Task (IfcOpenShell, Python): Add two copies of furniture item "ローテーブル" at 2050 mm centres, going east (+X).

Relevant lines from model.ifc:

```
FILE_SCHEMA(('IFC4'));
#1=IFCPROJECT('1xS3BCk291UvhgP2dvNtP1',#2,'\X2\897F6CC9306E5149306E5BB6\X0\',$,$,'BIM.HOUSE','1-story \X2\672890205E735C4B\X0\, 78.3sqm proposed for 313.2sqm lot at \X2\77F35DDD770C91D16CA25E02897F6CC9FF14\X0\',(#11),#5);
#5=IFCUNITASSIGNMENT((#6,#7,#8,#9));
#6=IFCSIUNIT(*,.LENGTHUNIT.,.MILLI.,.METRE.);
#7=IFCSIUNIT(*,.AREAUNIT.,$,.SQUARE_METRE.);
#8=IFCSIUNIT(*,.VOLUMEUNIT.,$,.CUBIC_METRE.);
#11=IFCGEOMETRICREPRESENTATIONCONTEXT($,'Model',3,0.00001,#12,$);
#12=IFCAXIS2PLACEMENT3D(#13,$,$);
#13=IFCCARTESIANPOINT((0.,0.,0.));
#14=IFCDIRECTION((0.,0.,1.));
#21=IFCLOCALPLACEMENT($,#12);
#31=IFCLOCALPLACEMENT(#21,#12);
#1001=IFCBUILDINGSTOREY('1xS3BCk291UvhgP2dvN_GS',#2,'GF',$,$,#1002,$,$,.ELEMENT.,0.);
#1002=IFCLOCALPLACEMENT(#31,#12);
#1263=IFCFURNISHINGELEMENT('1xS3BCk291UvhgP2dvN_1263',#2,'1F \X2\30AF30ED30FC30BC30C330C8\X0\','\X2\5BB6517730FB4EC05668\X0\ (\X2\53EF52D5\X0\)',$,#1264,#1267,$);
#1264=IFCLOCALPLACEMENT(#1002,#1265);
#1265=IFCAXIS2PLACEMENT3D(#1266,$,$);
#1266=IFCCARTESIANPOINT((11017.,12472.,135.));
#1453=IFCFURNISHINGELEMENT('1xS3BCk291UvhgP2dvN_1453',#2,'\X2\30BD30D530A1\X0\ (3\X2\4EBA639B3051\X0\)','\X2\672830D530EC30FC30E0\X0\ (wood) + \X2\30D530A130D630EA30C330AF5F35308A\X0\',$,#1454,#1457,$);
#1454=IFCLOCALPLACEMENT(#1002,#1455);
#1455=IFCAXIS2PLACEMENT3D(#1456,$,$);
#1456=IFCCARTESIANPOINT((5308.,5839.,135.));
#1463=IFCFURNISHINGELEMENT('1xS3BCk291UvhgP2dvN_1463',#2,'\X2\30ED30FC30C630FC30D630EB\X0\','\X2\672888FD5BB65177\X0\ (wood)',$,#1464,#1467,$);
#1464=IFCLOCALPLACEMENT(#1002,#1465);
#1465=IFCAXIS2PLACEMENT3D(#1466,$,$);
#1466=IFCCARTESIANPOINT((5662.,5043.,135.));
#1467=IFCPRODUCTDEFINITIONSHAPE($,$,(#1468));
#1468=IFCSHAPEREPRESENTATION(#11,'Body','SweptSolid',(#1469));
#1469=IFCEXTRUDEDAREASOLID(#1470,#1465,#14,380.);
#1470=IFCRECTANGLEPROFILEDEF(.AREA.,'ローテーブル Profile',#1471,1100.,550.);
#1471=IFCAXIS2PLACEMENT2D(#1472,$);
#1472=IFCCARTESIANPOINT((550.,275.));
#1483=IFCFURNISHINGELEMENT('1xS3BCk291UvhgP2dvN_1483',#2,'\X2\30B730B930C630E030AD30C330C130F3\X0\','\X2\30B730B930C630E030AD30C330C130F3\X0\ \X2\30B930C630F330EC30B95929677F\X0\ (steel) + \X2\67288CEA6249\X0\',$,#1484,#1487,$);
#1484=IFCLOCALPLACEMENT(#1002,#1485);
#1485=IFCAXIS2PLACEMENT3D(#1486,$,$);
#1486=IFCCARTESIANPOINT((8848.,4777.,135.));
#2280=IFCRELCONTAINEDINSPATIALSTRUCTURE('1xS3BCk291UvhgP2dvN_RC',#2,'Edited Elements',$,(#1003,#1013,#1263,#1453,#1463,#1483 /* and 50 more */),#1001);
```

```python
import numpy as np
import ifcopenshell
import ifcopenshell.api.geometry
import ifcopenshell.api.root
import ifcopenshell.util.element
import ifcopenshell.util.placement
import ifcopenshell.util.unit

model = ifcopenshell.open("model.ifc")
unit_scale = ifcopenshell.util.unit.calculate_unit_scale(model)


def reuse_history(source, copy):
    """copy_class also copies each property set's owner history, people and application; keep the originals."""
    for rel in copy.IsDefinedBy:
        if rel.is_a("IfcRelDefinesByProperties") and (history := rel.RelatingPropertyDefinition.OwnerHistory):
            rel.RelatingPropertyDefinition.OwnerHistory = source.OwnerHistory
            ifcopenshell.util.element.remove_deep2(model, history)


source = model.by_id(1463)
base = ifcopenshell.util.placement.get_local_placement(source.ObjectPlacement)
step = np.array([1.0, 0.0, 0.0]) * 2.05 / unit_scale

for i in range(1, 3):
    copy = ifcopenshell.api.root.copy_class(model, product=source)
    copy.Representation = ifcopenshell.util.element.copy_deep(
        model, source.Representation, exclude=["IfcGeometricRepresentationContext", "IfcRepresentationMap"]
    )
    reuse_history(source, copy)
    matrix = base.copy()
    matrix[:3, 3] += i * step
    print("added at", matrix[:3, 3].round(3) + 0.0)
    ifcopenshell.api.geometry.edit_object_placement(model, product=copy, matrix=matrix, is_si=False)

model.write("model_updated.ifc")
```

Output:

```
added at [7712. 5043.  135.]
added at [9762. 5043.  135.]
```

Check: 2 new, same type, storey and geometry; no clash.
